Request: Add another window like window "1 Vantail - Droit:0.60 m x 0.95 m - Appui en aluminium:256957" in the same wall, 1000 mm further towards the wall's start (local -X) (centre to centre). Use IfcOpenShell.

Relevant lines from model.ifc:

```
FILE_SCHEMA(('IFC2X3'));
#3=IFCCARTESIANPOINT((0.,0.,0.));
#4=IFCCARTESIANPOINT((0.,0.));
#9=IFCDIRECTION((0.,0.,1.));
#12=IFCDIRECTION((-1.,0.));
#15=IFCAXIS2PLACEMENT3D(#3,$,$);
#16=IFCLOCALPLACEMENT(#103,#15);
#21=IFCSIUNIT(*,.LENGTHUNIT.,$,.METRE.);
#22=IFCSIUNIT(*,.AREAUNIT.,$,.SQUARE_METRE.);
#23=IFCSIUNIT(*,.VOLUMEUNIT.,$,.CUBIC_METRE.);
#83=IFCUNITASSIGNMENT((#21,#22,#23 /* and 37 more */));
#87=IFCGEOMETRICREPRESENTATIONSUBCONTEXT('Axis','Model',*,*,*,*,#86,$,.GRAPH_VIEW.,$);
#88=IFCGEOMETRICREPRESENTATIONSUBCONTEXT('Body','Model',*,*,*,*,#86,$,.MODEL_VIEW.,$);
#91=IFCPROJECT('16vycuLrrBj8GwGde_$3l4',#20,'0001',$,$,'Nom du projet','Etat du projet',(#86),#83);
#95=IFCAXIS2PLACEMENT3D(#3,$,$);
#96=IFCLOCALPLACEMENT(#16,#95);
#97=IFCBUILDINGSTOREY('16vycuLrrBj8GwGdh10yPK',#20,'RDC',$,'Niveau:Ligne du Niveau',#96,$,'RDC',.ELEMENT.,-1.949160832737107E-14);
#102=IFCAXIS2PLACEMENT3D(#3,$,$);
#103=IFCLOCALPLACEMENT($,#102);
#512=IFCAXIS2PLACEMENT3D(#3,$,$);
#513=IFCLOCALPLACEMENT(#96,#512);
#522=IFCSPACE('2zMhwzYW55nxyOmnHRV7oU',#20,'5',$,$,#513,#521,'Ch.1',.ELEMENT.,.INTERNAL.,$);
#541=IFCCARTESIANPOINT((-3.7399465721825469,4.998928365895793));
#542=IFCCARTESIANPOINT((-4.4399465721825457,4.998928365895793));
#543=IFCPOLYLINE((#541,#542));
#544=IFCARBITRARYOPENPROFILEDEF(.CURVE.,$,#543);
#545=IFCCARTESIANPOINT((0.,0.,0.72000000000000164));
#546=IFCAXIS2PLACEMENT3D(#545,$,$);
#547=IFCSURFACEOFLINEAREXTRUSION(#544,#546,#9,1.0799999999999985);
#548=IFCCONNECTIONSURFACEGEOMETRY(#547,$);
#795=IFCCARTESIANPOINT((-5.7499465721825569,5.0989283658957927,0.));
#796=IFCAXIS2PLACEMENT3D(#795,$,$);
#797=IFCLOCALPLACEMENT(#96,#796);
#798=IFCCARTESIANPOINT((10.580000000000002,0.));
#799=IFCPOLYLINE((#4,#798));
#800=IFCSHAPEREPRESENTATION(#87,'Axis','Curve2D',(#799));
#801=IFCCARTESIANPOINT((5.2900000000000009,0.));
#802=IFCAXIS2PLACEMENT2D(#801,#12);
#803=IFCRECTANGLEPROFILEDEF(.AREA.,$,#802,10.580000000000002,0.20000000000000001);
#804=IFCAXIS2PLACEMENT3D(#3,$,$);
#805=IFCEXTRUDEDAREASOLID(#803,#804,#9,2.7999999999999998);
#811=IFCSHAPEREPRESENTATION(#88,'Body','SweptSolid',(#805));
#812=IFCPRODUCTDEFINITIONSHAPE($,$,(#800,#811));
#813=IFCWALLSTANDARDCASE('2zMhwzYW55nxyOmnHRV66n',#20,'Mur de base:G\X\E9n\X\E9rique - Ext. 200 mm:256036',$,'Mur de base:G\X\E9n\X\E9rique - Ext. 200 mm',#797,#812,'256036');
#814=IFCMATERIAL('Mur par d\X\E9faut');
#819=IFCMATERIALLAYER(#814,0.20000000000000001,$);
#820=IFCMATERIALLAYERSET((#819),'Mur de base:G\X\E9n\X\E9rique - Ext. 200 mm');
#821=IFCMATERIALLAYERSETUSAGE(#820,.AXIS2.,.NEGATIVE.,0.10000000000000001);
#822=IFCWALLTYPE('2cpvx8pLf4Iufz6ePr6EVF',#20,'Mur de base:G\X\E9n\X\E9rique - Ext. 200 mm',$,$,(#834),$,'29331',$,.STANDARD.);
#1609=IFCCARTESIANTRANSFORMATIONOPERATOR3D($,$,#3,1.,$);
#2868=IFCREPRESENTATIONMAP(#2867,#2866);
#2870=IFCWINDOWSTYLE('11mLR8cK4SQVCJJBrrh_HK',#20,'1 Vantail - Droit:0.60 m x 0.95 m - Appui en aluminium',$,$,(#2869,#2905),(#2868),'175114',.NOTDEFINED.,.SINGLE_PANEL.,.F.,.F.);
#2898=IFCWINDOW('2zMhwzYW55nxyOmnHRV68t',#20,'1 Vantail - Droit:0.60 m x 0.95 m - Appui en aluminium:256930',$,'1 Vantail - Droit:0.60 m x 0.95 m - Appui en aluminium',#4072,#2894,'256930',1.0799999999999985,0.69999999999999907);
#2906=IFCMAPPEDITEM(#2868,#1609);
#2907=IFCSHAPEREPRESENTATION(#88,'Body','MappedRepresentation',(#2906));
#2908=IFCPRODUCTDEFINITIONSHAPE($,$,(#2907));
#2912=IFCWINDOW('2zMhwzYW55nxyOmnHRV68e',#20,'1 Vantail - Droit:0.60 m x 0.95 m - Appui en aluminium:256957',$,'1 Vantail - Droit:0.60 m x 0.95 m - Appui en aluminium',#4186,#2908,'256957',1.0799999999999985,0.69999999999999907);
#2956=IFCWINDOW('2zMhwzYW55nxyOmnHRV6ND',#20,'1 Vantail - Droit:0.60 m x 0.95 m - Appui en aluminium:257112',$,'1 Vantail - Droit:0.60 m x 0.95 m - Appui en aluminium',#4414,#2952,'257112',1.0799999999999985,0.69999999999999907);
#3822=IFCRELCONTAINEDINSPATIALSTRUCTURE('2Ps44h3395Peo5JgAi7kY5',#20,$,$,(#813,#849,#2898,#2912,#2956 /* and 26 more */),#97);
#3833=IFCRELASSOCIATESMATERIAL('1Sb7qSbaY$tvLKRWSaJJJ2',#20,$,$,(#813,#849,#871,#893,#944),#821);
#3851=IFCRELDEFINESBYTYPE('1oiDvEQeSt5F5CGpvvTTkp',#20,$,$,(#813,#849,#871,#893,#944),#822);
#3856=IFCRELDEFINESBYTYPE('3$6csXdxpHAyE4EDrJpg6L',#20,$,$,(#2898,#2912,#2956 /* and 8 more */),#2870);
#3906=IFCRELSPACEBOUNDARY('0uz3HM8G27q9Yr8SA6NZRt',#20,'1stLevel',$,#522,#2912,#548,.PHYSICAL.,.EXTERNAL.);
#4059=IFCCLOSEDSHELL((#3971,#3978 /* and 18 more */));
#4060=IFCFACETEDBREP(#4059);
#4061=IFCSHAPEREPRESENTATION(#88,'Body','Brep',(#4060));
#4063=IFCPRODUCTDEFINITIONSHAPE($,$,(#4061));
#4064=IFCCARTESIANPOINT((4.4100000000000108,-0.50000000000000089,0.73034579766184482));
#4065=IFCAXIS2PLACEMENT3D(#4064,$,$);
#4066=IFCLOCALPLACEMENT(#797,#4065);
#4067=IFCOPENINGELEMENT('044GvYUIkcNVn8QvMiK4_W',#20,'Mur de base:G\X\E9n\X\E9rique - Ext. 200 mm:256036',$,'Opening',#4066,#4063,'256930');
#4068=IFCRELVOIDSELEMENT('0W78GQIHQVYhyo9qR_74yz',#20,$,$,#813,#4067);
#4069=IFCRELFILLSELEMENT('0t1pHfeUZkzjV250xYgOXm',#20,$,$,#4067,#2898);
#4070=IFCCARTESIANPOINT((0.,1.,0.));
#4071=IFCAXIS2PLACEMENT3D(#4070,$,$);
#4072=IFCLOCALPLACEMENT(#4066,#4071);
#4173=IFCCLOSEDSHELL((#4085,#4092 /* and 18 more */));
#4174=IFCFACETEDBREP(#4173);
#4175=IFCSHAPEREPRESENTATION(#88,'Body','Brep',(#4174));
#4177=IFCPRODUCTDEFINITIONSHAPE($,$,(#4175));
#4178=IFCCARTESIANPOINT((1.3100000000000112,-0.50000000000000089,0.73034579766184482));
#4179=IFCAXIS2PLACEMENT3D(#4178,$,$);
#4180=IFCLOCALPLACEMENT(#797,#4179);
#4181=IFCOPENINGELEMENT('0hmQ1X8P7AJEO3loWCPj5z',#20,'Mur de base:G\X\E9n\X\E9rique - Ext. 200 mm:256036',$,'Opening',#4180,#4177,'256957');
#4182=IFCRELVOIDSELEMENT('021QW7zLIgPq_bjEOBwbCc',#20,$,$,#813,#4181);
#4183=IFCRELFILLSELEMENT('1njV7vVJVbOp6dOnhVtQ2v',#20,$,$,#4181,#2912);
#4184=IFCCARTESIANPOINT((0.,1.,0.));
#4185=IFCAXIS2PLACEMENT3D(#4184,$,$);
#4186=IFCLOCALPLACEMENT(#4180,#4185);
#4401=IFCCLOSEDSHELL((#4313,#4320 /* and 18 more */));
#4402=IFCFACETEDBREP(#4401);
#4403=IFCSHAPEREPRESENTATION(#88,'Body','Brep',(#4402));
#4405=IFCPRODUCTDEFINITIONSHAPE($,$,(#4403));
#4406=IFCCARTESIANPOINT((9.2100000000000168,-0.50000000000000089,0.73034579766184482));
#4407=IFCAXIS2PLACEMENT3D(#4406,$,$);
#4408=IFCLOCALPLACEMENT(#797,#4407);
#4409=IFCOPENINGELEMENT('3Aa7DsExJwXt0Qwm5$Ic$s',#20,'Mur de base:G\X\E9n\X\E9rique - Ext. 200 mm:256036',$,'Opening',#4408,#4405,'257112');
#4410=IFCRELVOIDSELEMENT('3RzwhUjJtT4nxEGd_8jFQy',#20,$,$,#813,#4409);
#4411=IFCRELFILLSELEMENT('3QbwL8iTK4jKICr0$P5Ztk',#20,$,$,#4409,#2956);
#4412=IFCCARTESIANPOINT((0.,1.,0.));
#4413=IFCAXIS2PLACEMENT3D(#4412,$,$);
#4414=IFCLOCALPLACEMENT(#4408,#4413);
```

```python
import numpy as np
import ifcopenshell
import ifcopenshell.api.feature
import ifcopenshell.api.geometry
import ifcopenshell.api.root
import ifcopenshell.geom
import ifcopenshell.util.element
import ifcopenshell.util.placement
import ifcopenshell.util.shape
import ifcopenshell.util.unit

model = ifcopenshell.open("model.ifc")
unit_scale = ifcopenshell.util.unit.calculate_unit_scale(model)
settings = ifcopenshell.geom.settings()


def volume(element):
    """Net volume in cubic metres, openings subtracted."""
    shape = ifcopenshell.geom.create_shape(settings, element)
    return ifcopenshell.util.shape.get_volume(shape.geometry)


def reuse_history(source, copy):
    """copy_class also copies each property set's owner history, people and application; keep the originals."""
    for rel in copy.IsDefinedBy:
        if rel.is_a("IfcRelDefinesByProperties") and (history := rel.RelatingPropertyDefinition.OwnerHistory):
            rel.RelatingPropertyDefinition.OwnerHistory = source.OwnerHistory
            ifcopenshell.util.element.remove_deep2(model, history)


window = model.by_guid("2zMhwzYW55nxyOmnHRV68e")
opening = window.FillsVoids[0].RelatingOpeningElement
wall = opening.VoidsElements[0].RelatingBuildingElement
before = volume(wall)
shift = ifcopenshell.util.placement.get_local_placement(wall.ObjectPlacement)[:3, 0] * -1 / unit_scale

# copy_class copies the void relationship, type, container and properties, but no geometry.
new_opening = ifcopenshell.api.root.copy_class(model, product=opening)
new_opening.Representation = ifcopenshell.util.element.copy_deep(
    model, opening.Representation, exclude=["IfcGeometricRepresentationContext", "IfcRepresentationMap"]
)
new_opening.Name = "Mur de base:Générique - Ext. 200 mm"
new_opening.Tag = None
new_window = ifcopenshell.api.root.copy_class(model, product=window)
new_window.Representation = ifcopenshell.util.element.copy_deep(
    model, window.Representation, exclude=["IfcGeometricRepresentationContext", "IfcRepresentationMap"]
)
new_window.Name = "1 Vantail - Droit:0.60 m x 0.95 m - Appui en aluminium"
new_window.Tag = None
reuse_history(window, new_window)
fills = ifcopenshell.api.feature.add_filling(model, opening=new_opening, element=new_window)
fills.OwnerHistory = new_window.OwnerHistory  # required in IFC2X3

for old, new in ((opening, new_opening), (window, new_window)):
    matrix = ifcopenshell.util.placement.get_local_placement(old.ObjectPlacement)
    matrix[:3, 3] += shift
    ifcopenshell.api.geometry.edit_object_placement(model, product=new, matrix=matrix, is_si=False)

# The copied space boundaries still share their surfaces with the original.
for rel in new_window.ProvidesBoundaries:
    if rel.ConnectionGeometry:
        rel.ConnectionGeometry = ifcopenshell.util.element.copy_deep(model, rel.ConnectionGeometry)

# Space boundary surfaces are stored in each space's coordinates; move them too.
for rel in new_window.ProvidesBoundaries:
    if not rel.ConnectionGeometry:
        continue
    surface = rel.ConnectionGeometry.SurfaceOnRelatingElement
    space_matrix = ifcopenshell.util.placement.get_local_placement(rel.RelatingSpace.ObjectPlacement)
    point = np.array(surface.Position.Location.Coordinates) + space_matrix[:3, :3].T @ shift
    surface.Position = model.createIfcAxis2Placement3D(
        model.createIfcCartesianPoint(point.tolist()), surface.Position.Axis, surface.Position.RefDirection
    )

after = volume(wall)

print(f"wall volume {before:.3f} -> {after:.3f} m3")

model.write("model_edited.ifc")
```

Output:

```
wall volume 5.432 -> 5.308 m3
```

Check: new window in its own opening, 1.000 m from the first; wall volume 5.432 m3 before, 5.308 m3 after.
